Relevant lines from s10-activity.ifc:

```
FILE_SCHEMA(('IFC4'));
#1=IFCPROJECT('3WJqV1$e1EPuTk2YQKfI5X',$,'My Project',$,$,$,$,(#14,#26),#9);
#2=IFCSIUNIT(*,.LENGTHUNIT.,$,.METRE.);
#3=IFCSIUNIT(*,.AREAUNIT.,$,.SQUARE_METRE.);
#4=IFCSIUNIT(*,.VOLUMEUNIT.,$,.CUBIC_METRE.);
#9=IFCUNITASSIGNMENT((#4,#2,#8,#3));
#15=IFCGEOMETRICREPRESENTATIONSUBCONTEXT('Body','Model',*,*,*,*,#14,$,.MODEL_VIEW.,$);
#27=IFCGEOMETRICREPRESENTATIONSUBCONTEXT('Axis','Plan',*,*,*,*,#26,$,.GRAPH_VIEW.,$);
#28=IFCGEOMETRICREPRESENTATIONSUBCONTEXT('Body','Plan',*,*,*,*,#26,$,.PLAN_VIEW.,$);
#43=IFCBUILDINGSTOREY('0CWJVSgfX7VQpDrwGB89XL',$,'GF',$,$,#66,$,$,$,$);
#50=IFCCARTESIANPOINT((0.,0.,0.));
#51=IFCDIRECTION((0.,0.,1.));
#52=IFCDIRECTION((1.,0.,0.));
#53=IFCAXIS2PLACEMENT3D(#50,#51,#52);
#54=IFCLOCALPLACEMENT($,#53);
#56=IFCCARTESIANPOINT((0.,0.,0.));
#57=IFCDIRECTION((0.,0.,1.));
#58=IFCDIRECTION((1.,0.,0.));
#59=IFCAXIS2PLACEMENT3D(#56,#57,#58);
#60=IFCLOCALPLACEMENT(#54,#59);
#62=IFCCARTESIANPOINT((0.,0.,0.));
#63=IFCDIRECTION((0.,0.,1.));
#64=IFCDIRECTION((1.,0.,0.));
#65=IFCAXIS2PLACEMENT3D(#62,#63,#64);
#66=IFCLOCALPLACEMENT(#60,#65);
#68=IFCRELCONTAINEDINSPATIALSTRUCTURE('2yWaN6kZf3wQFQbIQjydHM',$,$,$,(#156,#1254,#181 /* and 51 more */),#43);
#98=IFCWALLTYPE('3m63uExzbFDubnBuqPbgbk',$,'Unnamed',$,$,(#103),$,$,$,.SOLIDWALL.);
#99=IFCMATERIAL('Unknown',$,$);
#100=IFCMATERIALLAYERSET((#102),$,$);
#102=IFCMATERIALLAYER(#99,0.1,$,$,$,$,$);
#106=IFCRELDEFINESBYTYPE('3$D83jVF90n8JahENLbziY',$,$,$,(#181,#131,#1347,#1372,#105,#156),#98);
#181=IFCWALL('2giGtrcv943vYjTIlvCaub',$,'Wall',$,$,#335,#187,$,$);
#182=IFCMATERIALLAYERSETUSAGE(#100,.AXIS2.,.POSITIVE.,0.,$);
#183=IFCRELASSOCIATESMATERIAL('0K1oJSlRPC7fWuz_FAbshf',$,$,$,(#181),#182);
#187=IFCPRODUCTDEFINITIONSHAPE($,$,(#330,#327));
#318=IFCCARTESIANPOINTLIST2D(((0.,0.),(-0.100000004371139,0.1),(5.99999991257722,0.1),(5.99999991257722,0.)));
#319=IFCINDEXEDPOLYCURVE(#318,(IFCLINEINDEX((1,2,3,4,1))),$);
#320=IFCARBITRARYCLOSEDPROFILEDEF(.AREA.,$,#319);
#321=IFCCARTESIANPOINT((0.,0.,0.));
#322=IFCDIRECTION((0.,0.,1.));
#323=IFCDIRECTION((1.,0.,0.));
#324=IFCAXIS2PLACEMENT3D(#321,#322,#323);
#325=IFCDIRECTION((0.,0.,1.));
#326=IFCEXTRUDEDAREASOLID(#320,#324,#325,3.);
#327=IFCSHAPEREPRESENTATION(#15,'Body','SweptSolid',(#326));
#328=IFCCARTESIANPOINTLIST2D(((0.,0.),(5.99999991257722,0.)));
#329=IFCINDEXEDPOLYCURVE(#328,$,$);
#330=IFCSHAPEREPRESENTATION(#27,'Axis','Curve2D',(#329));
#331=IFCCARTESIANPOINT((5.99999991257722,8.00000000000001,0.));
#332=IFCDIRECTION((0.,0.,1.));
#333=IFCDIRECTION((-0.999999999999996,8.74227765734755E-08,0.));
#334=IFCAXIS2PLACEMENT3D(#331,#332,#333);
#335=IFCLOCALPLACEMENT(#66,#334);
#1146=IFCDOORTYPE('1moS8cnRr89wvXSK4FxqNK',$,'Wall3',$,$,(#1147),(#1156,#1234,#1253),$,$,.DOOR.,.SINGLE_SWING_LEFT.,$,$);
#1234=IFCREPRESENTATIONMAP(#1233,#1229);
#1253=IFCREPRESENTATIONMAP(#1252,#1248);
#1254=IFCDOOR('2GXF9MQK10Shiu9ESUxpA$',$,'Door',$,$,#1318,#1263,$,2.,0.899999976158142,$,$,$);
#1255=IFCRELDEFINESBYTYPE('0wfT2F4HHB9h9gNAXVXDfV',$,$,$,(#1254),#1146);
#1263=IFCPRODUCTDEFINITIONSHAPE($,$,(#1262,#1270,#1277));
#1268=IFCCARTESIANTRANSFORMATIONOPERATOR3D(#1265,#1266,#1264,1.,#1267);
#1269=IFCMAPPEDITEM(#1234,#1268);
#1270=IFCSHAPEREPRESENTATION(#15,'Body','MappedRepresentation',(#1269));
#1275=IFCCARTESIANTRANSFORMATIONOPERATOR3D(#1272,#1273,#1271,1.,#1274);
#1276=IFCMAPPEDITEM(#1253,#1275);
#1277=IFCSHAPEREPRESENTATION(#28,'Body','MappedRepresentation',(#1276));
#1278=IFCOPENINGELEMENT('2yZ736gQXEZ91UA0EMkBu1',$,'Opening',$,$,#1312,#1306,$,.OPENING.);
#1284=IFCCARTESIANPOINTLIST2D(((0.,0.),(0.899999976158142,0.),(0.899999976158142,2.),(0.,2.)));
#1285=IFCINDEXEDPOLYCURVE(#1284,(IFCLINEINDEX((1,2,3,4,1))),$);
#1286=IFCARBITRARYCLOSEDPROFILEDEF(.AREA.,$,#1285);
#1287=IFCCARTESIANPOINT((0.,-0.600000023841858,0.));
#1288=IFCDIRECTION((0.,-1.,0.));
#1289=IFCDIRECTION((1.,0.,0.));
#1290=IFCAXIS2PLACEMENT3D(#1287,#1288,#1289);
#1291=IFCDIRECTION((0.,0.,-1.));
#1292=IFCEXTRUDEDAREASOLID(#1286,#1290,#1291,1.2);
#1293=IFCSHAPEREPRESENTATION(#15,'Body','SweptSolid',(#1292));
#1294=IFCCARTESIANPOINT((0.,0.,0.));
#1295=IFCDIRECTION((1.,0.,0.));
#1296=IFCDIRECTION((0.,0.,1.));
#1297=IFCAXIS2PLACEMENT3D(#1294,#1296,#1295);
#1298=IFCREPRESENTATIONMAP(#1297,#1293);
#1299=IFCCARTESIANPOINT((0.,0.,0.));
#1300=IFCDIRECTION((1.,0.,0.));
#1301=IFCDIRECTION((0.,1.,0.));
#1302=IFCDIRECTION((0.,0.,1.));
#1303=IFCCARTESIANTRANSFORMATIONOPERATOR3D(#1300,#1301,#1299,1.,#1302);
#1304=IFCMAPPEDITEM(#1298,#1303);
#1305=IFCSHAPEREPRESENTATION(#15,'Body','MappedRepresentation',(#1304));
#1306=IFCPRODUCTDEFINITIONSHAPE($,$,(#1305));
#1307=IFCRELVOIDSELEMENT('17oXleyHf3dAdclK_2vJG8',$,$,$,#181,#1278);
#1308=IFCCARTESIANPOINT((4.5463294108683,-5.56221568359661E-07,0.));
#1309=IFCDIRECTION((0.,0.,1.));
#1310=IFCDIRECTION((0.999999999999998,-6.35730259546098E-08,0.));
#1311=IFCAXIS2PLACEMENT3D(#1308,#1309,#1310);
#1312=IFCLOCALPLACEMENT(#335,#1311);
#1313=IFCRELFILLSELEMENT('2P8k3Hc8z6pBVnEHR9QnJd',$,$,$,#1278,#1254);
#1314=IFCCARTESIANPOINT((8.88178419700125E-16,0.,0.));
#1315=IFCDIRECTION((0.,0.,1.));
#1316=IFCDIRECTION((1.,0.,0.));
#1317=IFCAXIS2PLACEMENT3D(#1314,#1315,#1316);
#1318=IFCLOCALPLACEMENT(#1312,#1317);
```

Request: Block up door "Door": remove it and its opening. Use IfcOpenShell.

```python
import ifcopenshell
import ifcopenshell.api.feature
import ifcopenshell.api.root
import ifcopenshell.geom
import ifcopenshell.util.shape

model = ifcopenshell.open("s10-activity.ifc")
settings = ifcopenshell.geom.settings()


def volume(element):
    """Net volume in cubic metres, openings subtracted."""
    shape = ifcopenshell.geom.create_shape(settings, element)
    return ifcopenshell.util.shape.get_volume(shape.geometry)


door = model.by_guid("2GXF9MQK10Shiu9ESUxpA$")
opening = door.FillsVoids[0].RelatingOpeningElement
wall = opening.VoidsElements[0].RelatingBuildingElement
before = volume(wall)

ifcopenshell.api.root.remove_product(model, product=door)
ifcopenshell.api.feature.remove_feature(model, feature=opening)

after = volume(wall)

print(f"wall volume {before:.3f} -> {after:.3f} m3")

model.write("s10-activity_rev.ifc")
```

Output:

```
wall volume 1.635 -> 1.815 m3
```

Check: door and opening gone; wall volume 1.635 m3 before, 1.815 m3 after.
